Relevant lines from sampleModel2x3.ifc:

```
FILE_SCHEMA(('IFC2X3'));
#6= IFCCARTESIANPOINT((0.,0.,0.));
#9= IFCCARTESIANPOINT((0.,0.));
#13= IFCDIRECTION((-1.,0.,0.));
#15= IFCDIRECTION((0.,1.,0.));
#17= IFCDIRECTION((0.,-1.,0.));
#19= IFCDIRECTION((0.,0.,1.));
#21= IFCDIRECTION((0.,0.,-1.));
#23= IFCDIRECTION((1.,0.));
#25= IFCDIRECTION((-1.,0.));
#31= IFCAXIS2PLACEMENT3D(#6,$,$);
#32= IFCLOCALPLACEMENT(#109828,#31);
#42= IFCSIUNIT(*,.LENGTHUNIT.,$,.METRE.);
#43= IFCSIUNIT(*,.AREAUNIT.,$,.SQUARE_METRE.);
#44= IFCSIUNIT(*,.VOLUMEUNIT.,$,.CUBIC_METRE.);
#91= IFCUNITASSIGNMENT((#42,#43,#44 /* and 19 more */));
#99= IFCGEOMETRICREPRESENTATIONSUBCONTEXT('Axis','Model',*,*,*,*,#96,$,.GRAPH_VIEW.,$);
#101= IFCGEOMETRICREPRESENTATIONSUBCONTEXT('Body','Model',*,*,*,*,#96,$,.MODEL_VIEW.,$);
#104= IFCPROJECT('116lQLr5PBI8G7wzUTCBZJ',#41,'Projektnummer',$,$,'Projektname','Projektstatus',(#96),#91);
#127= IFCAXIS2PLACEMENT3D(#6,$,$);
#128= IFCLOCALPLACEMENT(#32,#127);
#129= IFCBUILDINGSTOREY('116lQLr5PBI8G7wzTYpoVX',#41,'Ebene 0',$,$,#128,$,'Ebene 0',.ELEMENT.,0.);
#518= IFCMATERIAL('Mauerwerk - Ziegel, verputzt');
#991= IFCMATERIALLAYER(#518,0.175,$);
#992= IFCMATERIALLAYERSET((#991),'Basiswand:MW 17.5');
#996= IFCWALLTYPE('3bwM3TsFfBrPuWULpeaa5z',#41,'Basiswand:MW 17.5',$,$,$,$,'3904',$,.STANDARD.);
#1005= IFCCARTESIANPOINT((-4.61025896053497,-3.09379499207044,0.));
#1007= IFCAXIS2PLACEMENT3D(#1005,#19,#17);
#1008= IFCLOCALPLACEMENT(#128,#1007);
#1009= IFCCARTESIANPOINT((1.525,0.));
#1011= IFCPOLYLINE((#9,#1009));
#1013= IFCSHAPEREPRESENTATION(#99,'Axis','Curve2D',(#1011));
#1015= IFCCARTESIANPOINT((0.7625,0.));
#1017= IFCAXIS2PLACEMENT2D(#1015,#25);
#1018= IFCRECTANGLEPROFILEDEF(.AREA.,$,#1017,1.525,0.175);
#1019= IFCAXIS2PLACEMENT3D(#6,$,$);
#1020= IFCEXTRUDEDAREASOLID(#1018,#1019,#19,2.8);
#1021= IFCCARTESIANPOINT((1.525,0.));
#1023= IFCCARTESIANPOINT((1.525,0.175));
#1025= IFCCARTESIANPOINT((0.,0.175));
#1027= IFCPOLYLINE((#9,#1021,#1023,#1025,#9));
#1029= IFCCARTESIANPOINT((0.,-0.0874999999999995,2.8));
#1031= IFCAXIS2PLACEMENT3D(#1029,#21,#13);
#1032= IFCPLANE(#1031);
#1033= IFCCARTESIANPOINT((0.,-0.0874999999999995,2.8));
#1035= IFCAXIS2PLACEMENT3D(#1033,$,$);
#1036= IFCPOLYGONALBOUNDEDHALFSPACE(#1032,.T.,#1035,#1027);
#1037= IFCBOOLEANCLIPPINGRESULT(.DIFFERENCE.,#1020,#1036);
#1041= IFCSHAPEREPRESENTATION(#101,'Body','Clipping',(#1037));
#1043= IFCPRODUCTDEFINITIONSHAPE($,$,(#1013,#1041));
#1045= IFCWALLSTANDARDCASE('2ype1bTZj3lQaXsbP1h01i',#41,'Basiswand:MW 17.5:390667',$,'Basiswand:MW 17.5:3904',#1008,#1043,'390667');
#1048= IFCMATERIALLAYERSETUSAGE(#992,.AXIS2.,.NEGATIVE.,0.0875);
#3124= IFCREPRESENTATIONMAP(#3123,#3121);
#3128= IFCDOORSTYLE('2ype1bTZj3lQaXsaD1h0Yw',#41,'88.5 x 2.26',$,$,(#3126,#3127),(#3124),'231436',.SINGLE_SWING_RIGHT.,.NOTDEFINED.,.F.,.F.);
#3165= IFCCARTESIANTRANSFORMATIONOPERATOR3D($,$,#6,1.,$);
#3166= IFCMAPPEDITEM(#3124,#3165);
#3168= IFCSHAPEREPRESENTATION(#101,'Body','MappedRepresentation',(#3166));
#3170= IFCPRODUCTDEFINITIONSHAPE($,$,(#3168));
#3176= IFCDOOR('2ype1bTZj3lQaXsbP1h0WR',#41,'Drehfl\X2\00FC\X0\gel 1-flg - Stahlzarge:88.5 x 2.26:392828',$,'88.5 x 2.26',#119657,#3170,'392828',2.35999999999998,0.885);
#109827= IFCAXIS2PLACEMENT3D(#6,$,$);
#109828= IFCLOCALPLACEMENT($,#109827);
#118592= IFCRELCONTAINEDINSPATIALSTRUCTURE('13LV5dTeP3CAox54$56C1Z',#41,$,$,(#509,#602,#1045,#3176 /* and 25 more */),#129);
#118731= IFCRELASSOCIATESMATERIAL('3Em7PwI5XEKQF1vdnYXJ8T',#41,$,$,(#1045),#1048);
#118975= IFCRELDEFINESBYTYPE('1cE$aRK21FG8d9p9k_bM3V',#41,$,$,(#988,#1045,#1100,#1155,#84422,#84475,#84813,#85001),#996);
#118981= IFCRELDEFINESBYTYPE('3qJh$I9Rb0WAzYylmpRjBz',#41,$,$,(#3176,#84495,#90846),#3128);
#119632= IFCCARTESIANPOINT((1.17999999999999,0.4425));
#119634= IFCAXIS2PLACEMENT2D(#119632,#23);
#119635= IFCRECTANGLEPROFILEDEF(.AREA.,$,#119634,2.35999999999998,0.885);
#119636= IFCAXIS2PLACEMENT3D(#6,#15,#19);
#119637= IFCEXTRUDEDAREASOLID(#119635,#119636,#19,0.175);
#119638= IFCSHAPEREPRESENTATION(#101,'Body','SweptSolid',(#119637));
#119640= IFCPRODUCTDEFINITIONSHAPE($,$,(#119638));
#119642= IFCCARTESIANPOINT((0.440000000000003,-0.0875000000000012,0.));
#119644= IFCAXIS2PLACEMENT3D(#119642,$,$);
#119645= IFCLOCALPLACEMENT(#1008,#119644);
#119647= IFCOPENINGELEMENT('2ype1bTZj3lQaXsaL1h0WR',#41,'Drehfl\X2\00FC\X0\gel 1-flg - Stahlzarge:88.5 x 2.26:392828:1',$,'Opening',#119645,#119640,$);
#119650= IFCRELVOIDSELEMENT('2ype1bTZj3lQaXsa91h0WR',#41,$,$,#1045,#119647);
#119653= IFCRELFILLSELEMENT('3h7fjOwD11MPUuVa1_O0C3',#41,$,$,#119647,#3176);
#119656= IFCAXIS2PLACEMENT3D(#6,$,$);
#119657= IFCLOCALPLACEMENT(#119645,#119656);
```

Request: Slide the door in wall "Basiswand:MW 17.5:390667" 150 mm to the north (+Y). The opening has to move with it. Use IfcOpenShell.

```python
import ifcopenshell
import ifcopenshell.api.geometry
import ifcopenshell.util.placement

model = ifcopenshell.open("sampleModel2x3.ifc")

door = model.by_id(3176)
opening = door.FillsVoids[0].RelatingOpeningElement
wall = opening.VoidsElements[0].RelatingBuildingElement

wall_matrix = ifcopenshell.util.placement.get_local_placement(wall.ObjectPlacement)
shift = wall_matrix[:3, 0] * -0.15
before = ifcopenshell.util.placement.get_local_placement(door.ObjectPlacement)[:3, 3].copy()

# The door is placed relative to its opening, so it follows when the opening moves.
matrix = ifcopenshell.util.placement.get_local_placement(opening.ObjectPlacement)
matrix[:3, 3] += shift
ifcopenshell.api.geometry.edit_object_placement(
    model, product=opening, matrix=matrix, is_si=False, should_transform_children=True
)

after = ifcopenshell.util.placement.get_local_placement(door.ObjectPlacement)[:3, 3]
print("door moved by", (after - before).round(3) + 0.0)

model.write("sampleModel2x3_edited.ifc")
```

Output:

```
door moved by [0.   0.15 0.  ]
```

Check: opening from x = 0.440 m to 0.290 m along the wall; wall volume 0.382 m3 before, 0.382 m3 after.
